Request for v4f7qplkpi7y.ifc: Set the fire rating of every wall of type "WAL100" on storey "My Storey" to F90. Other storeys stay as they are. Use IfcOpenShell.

First a look at what the model holds.

```python
import ifcopenshell
import ifcopenshell.util.element

model = ifcopenshell.open("v4f7qplkpi7y.ifc")
print(model.schema)
storey = next(s for s in model.by_type("IfcBuildingStorey") if s.Name == "My Storey")
walls = [e for e in ifcopenshell.util.element.get_decomposition(storey) if e.is_a("IfcWall")]
seen = {}
for e in walls:
    element_type = ifcopenshell.util.element.get_type(e)
    key = (element_type.Name if element_type != e and element_type else None, ifcopenshell.util.element.get_pset(e, "Pset_WallCommon", "FireRating"))
    seen[key] = seen.get(key, 0) + 1
for (name, value), count in sorted(seen.items(), key=str):
    print(count, "x", name, "|", value)
```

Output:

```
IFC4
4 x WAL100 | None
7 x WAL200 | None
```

```python
import ifcopenshell
import ifcopenshell.api.pset
import ifcopenshell.util.element

model = ifcopenshell.open("v4f7qplkpi7y.ifc")

storey = next(s for s in model.by_type("IfcBuildingStorey") if s.Name == "My Storey")
walls = [e for e in ifcopenshell.util.element.get_decomposition(storey) if e.is_a("IfcWall")]

count = 0
for e in walls:
    element_type = ifcopenshell.util.element.get_type(e)
    if element_type in (None, e) or element_type.Name != "WAL100":
        continue
    # add_pset returns the element's existing set when there is one.
    pset = ifcopenshell.api.pset.add_pset(model, product=e, name="Pset_WallCommon")
    ifcopenshell.api.pset.edit_pset(model, pset=pset, properties={"FireRating": "F90"})
    count += 1

print(count, "walls updated")

model.write("v4f7qplkpi7y_v2.ifc")
```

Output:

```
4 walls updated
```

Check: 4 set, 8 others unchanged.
